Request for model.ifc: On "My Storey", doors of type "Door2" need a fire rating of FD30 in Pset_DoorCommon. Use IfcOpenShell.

First a look at what the model holds.

```python
import ifcopenshell
import ifcopenshell.util.element

model = ifcopenshell.open("model.ifc")
print(model.schema)
storey = next(s for s in model.by_type("IfcBuildingStorey") if s.Name == "My Storey")
doors = [e for e in ifcopenshell.util.element.get_decomposition(storey) if e.is_a("IfcDoor")]
seen = {}
for e in doors:
    element_type = ifcopenshell.util.element.get_type(e)
    key = (element_type.Name if element_type != e and element_type else None, ifcopenshell.util.element.get_pset(e, "Pset_DoorCommon", "FireRating"))
    seen[key] = seen.get(key, 0) + 1
for (name, value), count in sorted(seen.items(), key=str):
    print(count, "x", name, "|", value)
```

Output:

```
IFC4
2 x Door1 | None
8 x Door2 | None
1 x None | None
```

```python
import ifcopenshell
import ifcopenshell.api.pset
import ifcopenshell.util.element

model = ifcopenshell.open("model.ifc")

storey = next(s for s in model.by_type("IfcBuildingStorey") if s.Name == "My Storey")
doors = [e for e in ifcopenshell.util.element.get_decomposition(storey) if e.is_a("IfcDoor")]

count = 0
for e in doors:
    element_type = ifcopenshell.util.element.get_type(e)
    if element_type in (None, e) or element_type.Name != "Door2":
        continue
    # add_pset returns the element's existing set when there is one.
    pset = ifcopenshell.api.pset.add_pset(model, product=e, name="Pset_DoorCommon")
    ifcopenshell.api.pset.edit_pset(model, pset=pset, properties={"FireRating": "FD30"})
    count += 1

print(count, "doors updated")

model.write("model_edited.ifc")
```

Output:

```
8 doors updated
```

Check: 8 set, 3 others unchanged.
